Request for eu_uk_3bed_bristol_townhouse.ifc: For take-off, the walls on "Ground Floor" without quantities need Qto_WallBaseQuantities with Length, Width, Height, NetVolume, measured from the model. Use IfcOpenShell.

First a look at what the model holds.

```python
import ifcopenshell
import ifcopenshell.util.element
import ifcopenshell.util.unit

model = ifcopenshell.open("eu_uk_3bed_bristol_townhouse.ifc")
print(model.schema)
for unit_type in ("LENGTHUNIT", "AREAUNIT", "VOLUMEUNIT"):
    print(unit_type, ifcopenshell.util.unit.calculate_unit_scale(model, unit_type))
storey = next(s for s in model.by_type("IfcBuildingStorey") if s.Name == "Ground Floor")
walls = [e for e in ifcopenshell.util.element.get_decomposition(storey) if e.is_a("IfcWall")]
for e in sorted(walls, key=lambda e: e.id()):
    print(e.id(), e.is_a(), e.Name, list(ifcopenshell.util.element.get_psets(e, qtos_only=True)), sep=" | ")
```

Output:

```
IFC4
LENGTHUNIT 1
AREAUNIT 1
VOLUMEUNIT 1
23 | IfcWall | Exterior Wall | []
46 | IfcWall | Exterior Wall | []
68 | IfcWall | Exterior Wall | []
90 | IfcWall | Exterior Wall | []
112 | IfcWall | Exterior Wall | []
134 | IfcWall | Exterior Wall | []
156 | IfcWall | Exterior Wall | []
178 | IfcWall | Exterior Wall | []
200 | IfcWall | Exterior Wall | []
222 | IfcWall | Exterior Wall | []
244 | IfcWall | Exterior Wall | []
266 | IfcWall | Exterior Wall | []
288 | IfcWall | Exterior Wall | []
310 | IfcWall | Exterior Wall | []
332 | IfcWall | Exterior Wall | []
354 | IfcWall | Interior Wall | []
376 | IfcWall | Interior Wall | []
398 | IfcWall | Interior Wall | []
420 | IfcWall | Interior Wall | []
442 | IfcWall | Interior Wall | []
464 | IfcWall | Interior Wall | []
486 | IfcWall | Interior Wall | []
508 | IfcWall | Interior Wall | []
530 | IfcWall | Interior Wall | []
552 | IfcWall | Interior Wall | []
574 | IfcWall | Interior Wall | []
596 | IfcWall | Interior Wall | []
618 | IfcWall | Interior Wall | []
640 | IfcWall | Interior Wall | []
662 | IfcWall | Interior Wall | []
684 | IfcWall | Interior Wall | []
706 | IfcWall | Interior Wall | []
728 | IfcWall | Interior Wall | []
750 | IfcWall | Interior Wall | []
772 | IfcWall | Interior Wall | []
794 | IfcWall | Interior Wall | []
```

```python
import ifcopenshell
import ifcopenshell.api.pset
import ifcopenshell.geom
import ifcopenshell.util.element
import ifcopenshell.util.shape
import ifcopenshell.util.unit

model = ifcopenshell.open("eu_uk_3bed_bristol_townhouse.ifc")
unit_scale = ifcopenshell.util.unit.calculate_unit_scale(model)
volume_scale = ifcopenshell.util.unit.calculate_unit_scale(model, "VOLUMEUNIT")
settings = ifcopenshell.geom.settings()

storey = next(s for s in model.by_type("IfcBuildingStorey") if s.Name == "Ground Floor")
walls = [e for e in ifcopenshell.util.element.get_decomposition(storey) if e.is_a("IfcWall")]

for e in sorted(walls, key=lambda e: e.id()):
    if ifcopenshell.util.element.get_psets(e, qtos_only=True, should_inherit=False):
        continue
    # Geometry comes back in metres, in the element's own axes.
    shape = ifcopenshell.geom.create_shape(settings, e)
    values = {
        "Length": ifcopenshell.util.shape.get_x(shape.geometry) / unit_scale,
        "Width": ifcopenshell.util.shape.get_y(shape.geometry) / unit_scale,
        "Height": ifcopenshell.util.shape.get_z(shape.geometry) / unit_scale,
        "NetVolume": ifcopenshell.util.shape.get_volume(shape.geometry) / volume_scale,
    }
    qto = ifcopenshell.api.pset.add_qto(model, product=e, name="Qto_WallBaseQuantities")
    ifcopenshell.api.pset.edit_qto(model, qto=qto, properties=values)
    print(e.id(), {k: round(v, 3) for k, v in values.items()})

model.write("eu_uk_3bed_bristol_townhouse_v2.ifc")
```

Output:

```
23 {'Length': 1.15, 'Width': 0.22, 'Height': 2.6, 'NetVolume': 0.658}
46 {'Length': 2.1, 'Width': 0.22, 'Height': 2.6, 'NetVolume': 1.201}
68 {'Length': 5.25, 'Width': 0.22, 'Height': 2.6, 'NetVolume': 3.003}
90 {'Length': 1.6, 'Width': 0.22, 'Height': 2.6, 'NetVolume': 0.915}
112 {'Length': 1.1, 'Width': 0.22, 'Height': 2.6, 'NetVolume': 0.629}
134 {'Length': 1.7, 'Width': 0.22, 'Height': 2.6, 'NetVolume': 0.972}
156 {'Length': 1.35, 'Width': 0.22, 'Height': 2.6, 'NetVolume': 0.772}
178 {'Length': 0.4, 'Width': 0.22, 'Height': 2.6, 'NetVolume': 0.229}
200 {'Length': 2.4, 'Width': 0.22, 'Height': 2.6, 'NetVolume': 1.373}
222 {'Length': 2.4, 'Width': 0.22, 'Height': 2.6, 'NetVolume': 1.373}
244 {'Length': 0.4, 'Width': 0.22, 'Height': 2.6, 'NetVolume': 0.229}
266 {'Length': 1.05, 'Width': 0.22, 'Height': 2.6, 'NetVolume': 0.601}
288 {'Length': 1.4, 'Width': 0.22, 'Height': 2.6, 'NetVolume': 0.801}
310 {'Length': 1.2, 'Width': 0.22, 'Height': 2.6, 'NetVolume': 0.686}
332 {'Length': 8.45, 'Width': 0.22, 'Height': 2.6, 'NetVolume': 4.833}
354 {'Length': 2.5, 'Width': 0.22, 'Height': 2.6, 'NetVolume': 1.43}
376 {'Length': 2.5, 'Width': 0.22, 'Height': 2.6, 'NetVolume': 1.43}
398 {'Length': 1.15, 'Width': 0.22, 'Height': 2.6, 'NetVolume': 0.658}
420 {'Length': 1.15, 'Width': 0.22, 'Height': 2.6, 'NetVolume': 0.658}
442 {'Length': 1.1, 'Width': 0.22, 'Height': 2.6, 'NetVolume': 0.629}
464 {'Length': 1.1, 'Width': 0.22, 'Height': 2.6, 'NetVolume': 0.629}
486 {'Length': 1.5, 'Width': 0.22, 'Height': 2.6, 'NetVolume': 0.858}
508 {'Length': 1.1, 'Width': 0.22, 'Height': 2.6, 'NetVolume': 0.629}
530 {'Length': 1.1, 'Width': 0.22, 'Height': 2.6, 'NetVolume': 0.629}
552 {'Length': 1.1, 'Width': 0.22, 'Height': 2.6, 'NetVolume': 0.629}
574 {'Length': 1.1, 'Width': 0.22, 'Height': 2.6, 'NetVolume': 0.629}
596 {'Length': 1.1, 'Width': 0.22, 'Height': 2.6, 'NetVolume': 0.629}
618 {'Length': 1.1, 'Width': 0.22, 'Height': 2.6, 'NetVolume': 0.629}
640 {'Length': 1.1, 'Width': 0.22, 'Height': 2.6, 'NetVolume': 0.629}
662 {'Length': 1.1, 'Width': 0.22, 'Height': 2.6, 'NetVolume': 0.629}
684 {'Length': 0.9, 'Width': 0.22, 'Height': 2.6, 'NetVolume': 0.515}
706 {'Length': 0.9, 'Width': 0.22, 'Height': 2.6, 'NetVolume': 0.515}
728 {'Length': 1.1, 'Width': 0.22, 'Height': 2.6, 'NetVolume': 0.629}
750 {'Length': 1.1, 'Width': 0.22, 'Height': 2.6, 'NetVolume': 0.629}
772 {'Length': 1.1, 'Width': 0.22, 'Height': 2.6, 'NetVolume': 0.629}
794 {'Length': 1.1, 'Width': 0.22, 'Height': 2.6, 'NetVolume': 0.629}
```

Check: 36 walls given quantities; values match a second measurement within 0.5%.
